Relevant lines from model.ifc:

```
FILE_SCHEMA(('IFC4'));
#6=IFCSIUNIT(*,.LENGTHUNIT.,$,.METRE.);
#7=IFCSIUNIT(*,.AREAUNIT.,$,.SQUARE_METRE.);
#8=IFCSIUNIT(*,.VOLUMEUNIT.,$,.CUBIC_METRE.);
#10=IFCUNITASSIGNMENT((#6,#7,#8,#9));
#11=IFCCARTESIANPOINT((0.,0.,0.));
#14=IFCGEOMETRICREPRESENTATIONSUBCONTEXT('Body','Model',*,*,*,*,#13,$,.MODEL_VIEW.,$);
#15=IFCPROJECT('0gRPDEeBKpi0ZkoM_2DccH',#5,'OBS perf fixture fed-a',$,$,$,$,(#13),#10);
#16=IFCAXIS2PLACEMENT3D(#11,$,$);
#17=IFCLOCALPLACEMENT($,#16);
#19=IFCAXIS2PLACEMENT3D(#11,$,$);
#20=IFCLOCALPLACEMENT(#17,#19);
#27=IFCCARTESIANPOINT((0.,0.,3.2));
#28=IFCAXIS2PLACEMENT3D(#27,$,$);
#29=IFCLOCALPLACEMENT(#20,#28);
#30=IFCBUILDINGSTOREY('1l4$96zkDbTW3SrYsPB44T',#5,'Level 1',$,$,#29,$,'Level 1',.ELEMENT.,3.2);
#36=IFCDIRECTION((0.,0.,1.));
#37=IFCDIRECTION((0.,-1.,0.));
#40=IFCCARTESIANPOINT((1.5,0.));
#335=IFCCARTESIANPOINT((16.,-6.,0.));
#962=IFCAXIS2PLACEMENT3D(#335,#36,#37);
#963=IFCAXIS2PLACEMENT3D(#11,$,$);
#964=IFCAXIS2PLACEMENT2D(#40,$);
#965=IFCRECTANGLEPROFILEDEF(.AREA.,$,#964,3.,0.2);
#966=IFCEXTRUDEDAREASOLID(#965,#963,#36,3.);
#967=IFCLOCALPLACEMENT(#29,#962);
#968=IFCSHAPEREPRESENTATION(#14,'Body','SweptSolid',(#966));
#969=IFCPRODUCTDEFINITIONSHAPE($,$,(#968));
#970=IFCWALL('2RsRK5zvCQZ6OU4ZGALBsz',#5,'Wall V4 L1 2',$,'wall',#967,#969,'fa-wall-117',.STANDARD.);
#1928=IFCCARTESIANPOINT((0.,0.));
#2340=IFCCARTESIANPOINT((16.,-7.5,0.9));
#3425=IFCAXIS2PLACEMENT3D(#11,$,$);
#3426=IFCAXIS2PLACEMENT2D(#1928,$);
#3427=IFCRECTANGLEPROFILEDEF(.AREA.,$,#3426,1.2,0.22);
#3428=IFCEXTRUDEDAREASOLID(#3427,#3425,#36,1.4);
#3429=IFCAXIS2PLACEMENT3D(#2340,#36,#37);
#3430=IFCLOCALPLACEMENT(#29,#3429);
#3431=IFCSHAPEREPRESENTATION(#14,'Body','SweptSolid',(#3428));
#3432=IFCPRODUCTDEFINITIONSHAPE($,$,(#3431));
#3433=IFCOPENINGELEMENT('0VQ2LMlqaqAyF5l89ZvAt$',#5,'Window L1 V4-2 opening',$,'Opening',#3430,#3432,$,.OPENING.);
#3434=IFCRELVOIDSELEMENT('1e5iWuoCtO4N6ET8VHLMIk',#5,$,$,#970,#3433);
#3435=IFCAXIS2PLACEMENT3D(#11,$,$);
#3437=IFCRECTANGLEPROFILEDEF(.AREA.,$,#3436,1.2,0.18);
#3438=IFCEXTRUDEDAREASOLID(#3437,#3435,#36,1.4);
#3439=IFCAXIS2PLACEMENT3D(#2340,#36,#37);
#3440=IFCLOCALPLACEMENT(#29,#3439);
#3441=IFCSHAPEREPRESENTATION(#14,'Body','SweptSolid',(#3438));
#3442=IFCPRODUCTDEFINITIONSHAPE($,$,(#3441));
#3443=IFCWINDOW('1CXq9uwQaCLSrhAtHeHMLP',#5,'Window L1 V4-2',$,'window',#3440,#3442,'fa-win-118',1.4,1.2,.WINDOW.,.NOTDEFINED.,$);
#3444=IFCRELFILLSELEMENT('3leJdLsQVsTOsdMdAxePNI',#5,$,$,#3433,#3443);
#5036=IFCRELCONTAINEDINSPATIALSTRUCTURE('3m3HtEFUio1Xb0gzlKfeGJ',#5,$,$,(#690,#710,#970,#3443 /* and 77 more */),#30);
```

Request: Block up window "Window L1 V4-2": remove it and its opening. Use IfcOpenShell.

```python
import ifcopenshell
import ifcopenshell.api.feature
import ifcopenshell.api.root
import ifcopenshell.geom
import ifcopenshell.util.shape

model = ifcopenshell.open("model.ifc")
settings = ifcopenshell.geom.settings()


def volume(element):
    """Net volume in cubic metres, openings subtracted."""
    shape = ifcopenshell.geom.create_shape(settings, element)
    return ifcopenshell.util.shape.get_volume(shape.geometry)


window = model.by_guid("1CXq9uwQaCLSrhAtHeHMLP")
opening = window.FillsVoids[0].RelatingOpeningElement
wall = opening.VoidsElements[0].RelatingBuildingElement
before = volume(wall)

ifcopenshell.api.root.remove_product(model, product=window)
ifcopenshell.api.feature.remove_feature(model, feature=opening)

after = volume(wall)

print(f"wall volume {before:.3f} -> {after:.3f} m3")

model.write("model_edited.ifc")
```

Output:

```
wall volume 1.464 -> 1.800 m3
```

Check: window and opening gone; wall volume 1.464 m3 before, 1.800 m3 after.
